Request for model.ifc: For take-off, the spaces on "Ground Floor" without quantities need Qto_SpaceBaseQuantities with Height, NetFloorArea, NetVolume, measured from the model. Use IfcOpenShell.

First a look at what the model holds.

```python
import ifcopenshell
import ifcopenshell.util.element
import ifcopenshell.util.unit

model = ifcopenshell.open("model.ifc")
print(model.schema)
for unit_type in ("LENGTHUNIT", "AREAUNIT", "VOLUMEUNIT"):
    print(unit_type, ifcopenshell.util.unit.calculate_unit_scale(model, unit_type))
storey = next(s for s in model.by_type("IfcBuildingStorey") if s.Name == "Ground Floor")
spaces = [e for e in ifcopenshell.util.element.get_decomposition(storey) if e.is_a("IfcSpace")]
for e in sorted(spaces, key=lambda e: e.id()):
    print(e.id(), e.is_a(), e.Name, list(ifcopenshell.util.element.get_psets(e, qtos_only=True)), sep=" | ")
```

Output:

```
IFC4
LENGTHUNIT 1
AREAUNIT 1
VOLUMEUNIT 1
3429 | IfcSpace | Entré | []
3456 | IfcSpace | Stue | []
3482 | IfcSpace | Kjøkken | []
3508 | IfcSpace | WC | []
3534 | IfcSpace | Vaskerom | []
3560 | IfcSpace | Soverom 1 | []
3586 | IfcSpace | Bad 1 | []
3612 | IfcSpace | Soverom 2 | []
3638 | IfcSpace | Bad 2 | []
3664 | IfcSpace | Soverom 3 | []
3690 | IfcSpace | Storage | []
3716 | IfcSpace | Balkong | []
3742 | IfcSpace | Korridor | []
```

```python
import ifcopenshell
import ifcopenshell.api.pset
import ifcopenshell.geom
import ifcopenshell.util.element
import ifcopenshell.util.shape
import ifcopenshell.util.unit

model = ifcopenshell.open("model.ifc")
unit_scale = ifcopenshell.util.unit.calculate_unit_scale(model)
area_scale = ifcopenshell.util.unit.calculate_unit_scale(model, "AREAUNIT")
volume_scale = ifcopenshell.util.unit.calculate_unit_scale(model, "VOLUMEUNIT")
settings = ifcopenshell.geom.settings()

storey = next(s for s in model.by_type("IfcBuildingStorey") if s.Name == "Ground Floor")
spaces = [e for e in ifcopenshell.util.element.get_decomposition(storey) if e.is_a("IfcSpace")]

for e in sorted(spaces, key=lambda e: e.id()):
    if ifcopenshell.util.element.get_psets(e, qtos_only=True, should_inherit=False):
        continue
    # Geometry comes back in metres, in the element's own axes.
    shape = ifcopenshell.geom.create_shape(settings, e)
    values = {
        "Height": ifcopenshell.util.shape.get_z(shape.geometry) / unit_scale,
        "NetFloorArea": ifcopenshell.util.shape.get_footprint_area(shape.geometry) / area_scale,
        "NetVolume": ifcopenshell.util.shape.get_volume(shape.geometry) / volume_scale,
    }
    qto = ifcopenshell.api.pset.add_qto(model, product=e, name="Qto_SpaceBaseQuantities")
    ifcopenshell.api.pset.edit_qto(model, qto=qto, properties=values)
    print(e.id(), {k: round(v, 3) for k, v in values.items()})

model.write("model_rev.ifc")
```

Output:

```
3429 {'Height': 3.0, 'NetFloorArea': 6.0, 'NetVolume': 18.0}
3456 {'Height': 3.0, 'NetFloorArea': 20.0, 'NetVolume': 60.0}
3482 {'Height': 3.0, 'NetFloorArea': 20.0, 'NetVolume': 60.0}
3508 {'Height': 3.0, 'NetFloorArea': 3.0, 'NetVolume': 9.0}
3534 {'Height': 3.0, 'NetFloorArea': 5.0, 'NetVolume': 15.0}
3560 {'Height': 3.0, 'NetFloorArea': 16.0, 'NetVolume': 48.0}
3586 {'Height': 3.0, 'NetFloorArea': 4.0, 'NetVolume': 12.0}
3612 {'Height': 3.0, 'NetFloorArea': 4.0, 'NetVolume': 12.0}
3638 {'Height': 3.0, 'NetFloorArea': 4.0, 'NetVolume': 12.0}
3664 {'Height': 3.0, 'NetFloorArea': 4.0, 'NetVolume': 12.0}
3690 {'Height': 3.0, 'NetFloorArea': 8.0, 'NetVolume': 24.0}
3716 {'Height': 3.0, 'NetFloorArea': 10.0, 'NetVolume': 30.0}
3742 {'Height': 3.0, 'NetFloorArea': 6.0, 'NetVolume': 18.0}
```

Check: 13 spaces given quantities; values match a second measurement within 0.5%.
